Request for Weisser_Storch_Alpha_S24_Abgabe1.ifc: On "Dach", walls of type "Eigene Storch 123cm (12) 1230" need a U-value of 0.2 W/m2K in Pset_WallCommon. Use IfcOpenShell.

First a look at what the model holds.

```python
import ifcopenshell
import ifcopenshell.util.element

model = ifcopenshell.open("Weisser_Storch_Alpha_S24_Abgabe1.ifc")
print(model.schema)
storey = next(s for s in model.by_type("IfcBuildingStorey") if s.Name == "Dach")
walls = [e for e in ifcopenshell.util.element.get_decomposition(storey) if e.is_a("IfcWall")]
seen = {}
for e in walls:
    element_type = ifcopenshell.util.element.get_type(e)
    key = (element_type.Name if element_type != e and element_type else None, ifcopenshell.util.element.get_pset(e, "Pset_WallCommon", "ThermalTransmittance"))
    seen[key] = seen.get(key, 0) + 1
for (name, value), count in sorted(seen.items(), key=str):
    print(count, "x", name, "|", value)
```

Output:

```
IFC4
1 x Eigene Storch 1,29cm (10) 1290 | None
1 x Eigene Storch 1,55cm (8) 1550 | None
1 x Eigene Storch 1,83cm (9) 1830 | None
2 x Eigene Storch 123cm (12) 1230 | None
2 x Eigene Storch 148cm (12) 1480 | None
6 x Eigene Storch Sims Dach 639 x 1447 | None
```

```python
import ifcopenshell
import ifcopenshell.api.pset
import ifcopenshell.util.element

model = ifcopenshell.open("Weisser_Storch_Alpha_S24_Abgabe1.ifc")

storey = next(s for s in model.by_type("IfcBuildingStorey") if s.Name == "Dach")
walls = [e for e in ifcopenshell.util.element.get_decomposition(storey) if e.is_a("IfcWall")]

count = 0
for e in walls:
    element_type = ifcopenshell.util.element.get_type(e)
    if element_type in (None, e) or element_type.Name != "Eigene Storch 123cm (12) 1230":
        continue
    # add_pset returns the element's existing set when there is one.
    pset = ifcopenshell.api.pset.add_pset(model, product=e, name="Pset_WallCommon")
    ifcopenshell.api.pset.edit_pset(model, pset=pset, properties={"ThermalTransmittance": 0.2})
    count += 1

print(count, "walls updated")

model.write("Weisser_Storch_Alpha_S24_Abgabe1_rev.ifc")
```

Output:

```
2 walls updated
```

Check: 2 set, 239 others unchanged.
